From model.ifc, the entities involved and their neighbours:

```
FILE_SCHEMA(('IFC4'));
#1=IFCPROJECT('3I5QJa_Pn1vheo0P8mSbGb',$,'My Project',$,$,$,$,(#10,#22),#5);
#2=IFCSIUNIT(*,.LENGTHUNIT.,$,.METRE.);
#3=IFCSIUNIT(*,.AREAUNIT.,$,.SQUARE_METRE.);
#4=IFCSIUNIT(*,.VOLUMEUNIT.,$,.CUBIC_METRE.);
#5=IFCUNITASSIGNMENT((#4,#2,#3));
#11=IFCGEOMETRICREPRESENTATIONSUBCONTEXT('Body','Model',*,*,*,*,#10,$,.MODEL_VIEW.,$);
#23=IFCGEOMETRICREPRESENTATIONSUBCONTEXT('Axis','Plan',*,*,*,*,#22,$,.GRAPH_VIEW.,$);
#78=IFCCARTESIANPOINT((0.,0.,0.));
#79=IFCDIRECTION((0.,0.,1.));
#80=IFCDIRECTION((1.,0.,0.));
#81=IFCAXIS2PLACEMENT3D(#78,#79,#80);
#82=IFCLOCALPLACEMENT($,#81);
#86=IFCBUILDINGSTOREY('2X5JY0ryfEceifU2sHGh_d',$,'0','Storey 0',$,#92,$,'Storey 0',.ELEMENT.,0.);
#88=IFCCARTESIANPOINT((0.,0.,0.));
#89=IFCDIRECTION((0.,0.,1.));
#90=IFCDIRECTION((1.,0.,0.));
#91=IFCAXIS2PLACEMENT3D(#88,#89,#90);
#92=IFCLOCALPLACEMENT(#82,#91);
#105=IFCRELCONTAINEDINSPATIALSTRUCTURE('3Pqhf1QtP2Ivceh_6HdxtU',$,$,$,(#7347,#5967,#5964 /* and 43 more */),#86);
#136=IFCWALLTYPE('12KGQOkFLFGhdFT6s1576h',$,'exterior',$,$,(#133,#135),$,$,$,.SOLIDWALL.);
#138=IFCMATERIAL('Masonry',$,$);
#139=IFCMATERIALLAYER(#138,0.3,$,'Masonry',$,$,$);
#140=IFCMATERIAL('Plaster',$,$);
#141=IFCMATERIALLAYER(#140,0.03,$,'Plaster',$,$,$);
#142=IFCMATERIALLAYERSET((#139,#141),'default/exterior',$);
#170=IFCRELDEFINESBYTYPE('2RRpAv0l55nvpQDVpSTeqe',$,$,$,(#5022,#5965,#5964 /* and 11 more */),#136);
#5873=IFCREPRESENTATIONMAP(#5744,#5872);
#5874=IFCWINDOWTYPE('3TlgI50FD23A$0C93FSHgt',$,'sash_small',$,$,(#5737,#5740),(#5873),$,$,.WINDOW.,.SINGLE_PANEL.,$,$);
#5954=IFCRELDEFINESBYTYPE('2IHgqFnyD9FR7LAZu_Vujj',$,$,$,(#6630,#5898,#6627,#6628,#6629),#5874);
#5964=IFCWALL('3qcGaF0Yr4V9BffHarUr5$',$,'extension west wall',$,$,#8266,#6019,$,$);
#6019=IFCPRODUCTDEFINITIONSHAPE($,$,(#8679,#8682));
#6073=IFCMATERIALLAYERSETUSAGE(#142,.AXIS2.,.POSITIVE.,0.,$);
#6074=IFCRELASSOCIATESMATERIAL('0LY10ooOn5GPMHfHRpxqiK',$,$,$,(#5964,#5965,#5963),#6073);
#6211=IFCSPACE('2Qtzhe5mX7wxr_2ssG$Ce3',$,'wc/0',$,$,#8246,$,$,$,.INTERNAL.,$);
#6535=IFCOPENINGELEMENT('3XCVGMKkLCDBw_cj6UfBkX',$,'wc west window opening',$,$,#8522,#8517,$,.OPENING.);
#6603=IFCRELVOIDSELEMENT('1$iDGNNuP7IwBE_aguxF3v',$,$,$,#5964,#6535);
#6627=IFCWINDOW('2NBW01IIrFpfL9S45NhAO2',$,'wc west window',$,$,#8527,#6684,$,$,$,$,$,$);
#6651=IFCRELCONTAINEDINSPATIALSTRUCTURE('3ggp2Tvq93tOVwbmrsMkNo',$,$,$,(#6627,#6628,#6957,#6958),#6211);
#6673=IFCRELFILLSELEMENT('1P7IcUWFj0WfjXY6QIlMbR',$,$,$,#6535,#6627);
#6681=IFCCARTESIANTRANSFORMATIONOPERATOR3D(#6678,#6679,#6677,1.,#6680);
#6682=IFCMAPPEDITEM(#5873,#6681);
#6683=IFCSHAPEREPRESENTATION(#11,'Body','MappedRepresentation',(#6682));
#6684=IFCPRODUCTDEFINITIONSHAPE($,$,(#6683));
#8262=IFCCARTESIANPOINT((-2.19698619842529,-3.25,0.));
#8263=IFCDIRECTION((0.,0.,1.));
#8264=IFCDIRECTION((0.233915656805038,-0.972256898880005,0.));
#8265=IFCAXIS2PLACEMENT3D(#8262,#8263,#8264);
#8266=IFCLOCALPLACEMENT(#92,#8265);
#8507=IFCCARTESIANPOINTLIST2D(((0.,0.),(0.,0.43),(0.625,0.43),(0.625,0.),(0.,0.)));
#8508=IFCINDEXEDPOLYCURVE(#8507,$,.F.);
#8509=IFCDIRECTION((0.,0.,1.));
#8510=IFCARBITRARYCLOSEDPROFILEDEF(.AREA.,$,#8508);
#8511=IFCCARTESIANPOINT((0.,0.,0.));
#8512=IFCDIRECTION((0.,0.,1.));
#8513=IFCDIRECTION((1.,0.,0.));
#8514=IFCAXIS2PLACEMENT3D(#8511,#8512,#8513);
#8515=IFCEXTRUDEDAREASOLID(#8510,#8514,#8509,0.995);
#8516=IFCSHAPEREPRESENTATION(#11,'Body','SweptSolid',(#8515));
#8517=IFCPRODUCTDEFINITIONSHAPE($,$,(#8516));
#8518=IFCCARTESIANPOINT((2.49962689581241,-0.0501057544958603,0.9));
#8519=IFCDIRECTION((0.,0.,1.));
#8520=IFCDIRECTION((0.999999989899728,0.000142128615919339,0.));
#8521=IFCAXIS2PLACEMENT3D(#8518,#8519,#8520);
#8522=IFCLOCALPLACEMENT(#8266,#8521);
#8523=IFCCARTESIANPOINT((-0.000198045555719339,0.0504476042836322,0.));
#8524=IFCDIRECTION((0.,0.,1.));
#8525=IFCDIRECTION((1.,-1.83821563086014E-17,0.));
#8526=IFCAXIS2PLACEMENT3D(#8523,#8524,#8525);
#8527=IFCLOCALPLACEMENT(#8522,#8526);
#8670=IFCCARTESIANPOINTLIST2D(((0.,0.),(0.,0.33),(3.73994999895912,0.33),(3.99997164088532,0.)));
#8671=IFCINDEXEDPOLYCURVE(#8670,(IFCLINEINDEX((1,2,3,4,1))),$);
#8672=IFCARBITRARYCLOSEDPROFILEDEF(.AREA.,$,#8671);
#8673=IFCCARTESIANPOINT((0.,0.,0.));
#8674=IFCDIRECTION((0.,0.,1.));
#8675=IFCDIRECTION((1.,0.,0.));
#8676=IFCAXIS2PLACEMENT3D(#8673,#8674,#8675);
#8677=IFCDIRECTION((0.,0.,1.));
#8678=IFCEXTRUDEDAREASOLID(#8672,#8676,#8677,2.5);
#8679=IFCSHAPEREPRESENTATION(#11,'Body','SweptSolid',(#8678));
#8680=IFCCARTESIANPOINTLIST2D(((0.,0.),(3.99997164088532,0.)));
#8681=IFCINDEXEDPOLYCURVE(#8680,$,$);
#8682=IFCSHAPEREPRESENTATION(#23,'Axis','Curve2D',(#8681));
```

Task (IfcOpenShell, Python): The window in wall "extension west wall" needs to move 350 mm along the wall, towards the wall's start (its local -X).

```python
import ifcopenshell
import ifcopenshell.api.geometry
import ifcopenshell.util.placement
import ifcopenshell.util.unit

model = ifcopenshell.open("model.ifc")
unit_scale = ifcopenshell.util.unit.calculate_unit_scale(model)

window = model.by_guid("2NBW01IIrFpfL9S45NhAO2")
opening = window.FillsVoids[0].RelatingOpeningElement
wall = opening.VoidsElements[0].RelatingBuildingElement

wall_matrix = ifcopenshell.util.placement.get_local_placement(wall.ObjectPlacement)
shift = wall_matrix[:3, 0] * -0.35 / unit_scale
before = ifcopenshell.util.placement.get_local_placement(window.ObjectPlacement)[:3, 3].copy()

# The window is placed relative to its opening, so it follows when the opening moves.
matrix = ifcopenshell.util.placement.get_local_placement(opening.ObjectPlacement)
matrix[:3, 3] += shift
ifcopenshell.api.geometry.edit_object_placement(
    model, product=opening, matrix=matrix, is_si=False, should_transform_children=True
)

after = ifcopenshell.util.placement.get_local_placement(window.ObjectPlacement)[:3, 3]
print("window moved by", (after - before).round(3) + 0.0)

model.write("model_updated.ifc")
```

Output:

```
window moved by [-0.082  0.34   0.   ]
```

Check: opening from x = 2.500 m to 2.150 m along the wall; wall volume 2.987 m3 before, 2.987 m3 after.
